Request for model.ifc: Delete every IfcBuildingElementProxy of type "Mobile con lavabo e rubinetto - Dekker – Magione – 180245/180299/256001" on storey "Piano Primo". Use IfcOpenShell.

First a look at what the model holds.

```python
import ifcopenshell
import ifcopenshell.util.element

model = ifcopenshell.open("model.ifc")
print(model.schema)
storey = next(s for s in model.by_type("IfcBuildingStorey") if s.Name == "Piano Primo")
proxies = [e for e in ifcopenshell.util.element.get_decomposition(storey) if e.is_a("IfcBuildingElementProxy")]
seen = {}
for e in proxies:
    element_type = ifcopenshell.util.element.get_type(e)
    name = element_type.Name if element_type not in (None, e) else None
    seen[name] = seen.get(name, 0) + 1
for name, count in sorted(seen.items(), key=str):
    print(count, "x", name)
```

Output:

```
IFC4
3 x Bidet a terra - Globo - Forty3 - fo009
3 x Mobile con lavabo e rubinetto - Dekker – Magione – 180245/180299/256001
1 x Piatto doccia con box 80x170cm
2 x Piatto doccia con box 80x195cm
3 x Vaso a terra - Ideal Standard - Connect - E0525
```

```python
import ifcopenshell
import ifcopenshell.api.root
import ifcopenshell.util.element

model = ifcopenshell.open("model.ifc")

storey = next(s for s in model.by_type("IfcBuildingStorey") if s.Name == "Piano Primo")
proxies = [e for e in ifcopenshell.util.element.get_decomposition(storey) if e.is_a("IfcBuildingElementProxy")]
targets = [e for e in proxies if (t := ifcopenshell.util.element.get_type(e)) not in (None, e) and t.Name == "Mobile con lavabo e rubinetto - Dekker – Magione – 180245/180299/256001"]

for e in targets:
    ifcopenshell.api.root.remove_product(model, product=e)
print(len(targets), "removed")

model.write("model_edited.ifc")
```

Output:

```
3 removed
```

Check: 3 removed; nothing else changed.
